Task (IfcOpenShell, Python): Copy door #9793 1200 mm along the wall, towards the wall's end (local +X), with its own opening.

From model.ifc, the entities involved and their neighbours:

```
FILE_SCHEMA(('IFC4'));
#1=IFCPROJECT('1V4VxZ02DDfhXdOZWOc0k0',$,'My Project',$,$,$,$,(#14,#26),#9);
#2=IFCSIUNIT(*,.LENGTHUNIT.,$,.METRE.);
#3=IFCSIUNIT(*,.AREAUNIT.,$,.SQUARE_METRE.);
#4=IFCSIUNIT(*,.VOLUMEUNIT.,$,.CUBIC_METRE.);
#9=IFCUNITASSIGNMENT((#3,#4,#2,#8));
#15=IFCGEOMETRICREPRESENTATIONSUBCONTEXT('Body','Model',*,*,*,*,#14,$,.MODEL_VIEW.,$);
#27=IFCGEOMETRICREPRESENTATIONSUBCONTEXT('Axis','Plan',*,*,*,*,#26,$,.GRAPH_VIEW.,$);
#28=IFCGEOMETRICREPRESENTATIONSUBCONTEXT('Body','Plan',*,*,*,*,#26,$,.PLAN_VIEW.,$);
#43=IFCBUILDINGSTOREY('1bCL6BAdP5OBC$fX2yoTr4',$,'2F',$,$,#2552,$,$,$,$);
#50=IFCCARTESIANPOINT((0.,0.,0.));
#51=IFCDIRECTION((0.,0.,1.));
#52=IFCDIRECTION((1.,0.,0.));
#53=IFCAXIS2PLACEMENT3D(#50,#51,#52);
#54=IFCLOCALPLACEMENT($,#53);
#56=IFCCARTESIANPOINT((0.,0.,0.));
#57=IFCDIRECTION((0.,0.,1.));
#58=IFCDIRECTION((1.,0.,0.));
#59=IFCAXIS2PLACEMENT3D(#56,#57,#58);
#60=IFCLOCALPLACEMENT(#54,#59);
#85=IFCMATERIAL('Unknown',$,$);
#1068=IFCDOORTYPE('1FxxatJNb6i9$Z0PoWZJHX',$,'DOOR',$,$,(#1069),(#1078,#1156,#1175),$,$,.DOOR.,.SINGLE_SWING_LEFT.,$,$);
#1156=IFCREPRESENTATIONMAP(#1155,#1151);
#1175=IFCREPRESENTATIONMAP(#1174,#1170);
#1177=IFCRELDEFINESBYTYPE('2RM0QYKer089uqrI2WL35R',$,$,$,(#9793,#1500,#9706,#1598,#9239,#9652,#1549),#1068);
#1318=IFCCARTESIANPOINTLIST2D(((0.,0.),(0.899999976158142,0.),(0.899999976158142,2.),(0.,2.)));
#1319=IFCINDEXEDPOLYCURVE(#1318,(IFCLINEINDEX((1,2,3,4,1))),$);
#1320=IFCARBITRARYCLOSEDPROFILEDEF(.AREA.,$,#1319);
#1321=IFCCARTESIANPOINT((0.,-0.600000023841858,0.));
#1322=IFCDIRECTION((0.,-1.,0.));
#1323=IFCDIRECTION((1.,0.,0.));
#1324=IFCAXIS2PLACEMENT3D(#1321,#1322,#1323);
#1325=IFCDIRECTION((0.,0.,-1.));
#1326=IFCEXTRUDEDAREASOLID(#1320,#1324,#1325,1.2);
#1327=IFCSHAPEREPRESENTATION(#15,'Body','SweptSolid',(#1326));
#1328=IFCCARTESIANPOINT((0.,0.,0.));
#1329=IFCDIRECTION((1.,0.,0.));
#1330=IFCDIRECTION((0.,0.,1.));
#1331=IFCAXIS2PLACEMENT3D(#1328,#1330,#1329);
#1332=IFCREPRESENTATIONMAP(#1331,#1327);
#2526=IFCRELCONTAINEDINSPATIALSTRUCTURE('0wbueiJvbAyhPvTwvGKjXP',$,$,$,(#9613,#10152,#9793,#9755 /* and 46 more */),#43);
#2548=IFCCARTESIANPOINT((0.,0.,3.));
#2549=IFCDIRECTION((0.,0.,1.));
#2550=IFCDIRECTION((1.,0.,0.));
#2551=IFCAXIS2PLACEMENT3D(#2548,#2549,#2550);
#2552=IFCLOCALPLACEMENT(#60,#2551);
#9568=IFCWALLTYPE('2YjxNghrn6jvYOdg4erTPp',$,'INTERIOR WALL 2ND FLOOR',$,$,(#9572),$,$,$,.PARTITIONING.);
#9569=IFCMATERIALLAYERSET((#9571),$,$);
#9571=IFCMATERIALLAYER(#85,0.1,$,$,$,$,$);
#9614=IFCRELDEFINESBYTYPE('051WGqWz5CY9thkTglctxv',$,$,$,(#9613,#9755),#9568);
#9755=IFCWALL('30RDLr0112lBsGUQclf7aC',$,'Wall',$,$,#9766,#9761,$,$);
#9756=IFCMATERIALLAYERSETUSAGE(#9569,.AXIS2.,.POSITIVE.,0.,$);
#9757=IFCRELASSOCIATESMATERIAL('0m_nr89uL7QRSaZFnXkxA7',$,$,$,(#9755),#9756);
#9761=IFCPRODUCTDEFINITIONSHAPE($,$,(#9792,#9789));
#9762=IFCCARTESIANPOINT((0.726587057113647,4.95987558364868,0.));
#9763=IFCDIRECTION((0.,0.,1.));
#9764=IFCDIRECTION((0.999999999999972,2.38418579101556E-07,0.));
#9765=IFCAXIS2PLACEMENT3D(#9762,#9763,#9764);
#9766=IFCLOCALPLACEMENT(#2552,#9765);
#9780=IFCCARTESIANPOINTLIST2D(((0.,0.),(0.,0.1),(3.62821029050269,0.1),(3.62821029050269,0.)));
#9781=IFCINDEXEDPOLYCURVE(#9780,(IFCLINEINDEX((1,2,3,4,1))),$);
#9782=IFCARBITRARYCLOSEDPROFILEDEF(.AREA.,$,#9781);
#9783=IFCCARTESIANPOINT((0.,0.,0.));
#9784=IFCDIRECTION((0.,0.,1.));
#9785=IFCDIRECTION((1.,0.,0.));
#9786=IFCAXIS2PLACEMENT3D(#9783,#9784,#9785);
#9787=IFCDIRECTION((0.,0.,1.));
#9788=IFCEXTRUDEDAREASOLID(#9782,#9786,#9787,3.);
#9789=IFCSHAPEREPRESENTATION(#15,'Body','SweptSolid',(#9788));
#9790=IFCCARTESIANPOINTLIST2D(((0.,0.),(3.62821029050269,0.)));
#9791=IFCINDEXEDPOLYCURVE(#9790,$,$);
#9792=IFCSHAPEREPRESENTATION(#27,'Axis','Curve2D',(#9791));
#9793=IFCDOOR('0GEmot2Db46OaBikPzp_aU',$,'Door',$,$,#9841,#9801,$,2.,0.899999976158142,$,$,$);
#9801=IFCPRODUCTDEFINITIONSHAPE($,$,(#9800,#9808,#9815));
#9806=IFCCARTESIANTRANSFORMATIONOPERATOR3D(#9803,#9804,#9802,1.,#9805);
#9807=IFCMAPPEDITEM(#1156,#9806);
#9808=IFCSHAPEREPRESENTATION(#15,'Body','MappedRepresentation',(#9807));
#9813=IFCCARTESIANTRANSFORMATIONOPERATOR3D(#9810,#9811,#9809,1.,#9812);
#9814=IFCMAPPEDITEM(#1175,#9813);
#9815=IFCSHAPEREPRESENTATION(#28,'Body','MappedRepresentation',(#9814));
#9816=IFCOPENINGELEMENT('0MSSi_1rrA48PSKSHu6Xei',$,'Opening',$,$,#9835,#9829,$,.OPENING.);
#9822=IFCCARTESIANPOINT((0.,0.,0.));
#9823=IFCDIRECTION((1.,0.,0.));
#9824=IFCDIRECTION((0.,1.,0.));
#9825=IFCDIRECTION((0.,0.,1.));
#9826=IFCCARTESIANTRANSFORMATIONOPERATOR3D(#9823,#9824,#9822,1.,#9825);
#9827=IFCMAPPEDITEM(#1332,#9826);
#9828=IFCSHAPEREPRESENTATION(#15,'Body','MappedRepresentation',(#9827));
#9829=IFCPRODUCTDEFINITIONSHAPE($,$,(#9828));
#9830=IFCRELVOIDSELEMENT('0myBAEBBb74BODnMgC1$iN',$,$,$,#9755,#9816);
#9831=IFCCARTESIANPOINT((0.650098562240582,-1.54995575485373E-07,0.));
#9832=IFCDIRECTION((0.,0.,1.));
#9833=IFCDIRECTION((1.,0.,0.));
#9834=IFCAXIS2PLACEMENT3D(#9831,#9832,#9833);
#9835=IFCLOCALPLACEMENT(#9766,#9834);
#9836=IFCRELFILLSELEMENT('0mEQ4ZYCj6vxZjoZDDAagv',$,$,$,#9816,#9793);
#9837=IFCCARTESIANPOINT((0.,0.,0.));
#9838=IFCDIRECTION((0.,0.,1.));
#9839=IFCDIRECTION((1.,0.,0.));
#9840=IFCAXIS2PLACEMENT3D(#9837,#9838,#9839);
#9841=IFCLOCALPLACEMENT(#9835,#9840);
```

```python
import ifcopenshell
import ifcopenshell.api.feature
import ifcopenshell.api.geometry
import ifcopenshell.api.root
import ifcopenshell.geom
import ifcopenshell.util.element
import ifcopenshell.util.placement
import ifcopenshell.util.shape

model = ifcopenshell.open("model.ifc")
settings = ifcopenshell.geom.settings()


def volume(element):
    """Net volume in cubic metres, openings subtracted."""
    shape = ifcopenshell.geom.create_shape(settings, element)
    return ifcopenshell.util.shape.get_volume(shape.geometry)


door = model.by_guid("0GEmot2Db46OaBikPzp_aU")
opening = door.FillsVoids[0].RelatingOpeningElement
wall = opening.VoidsElements[0].RelatingBuildingElement
before = volume(wall)
shift = ifcopenshell.util.placement.get_local_placement(wall.ObjectPlacement)[:3, 0] * 1.2

# copy_class copies the void relationship, type, container and properties, but no geometry.
new_opening = ifcopenshell.api.root.copy_class(model, product=opening)
new_opening.Representation = ifcopenshell.util.element.copy_deep(
    model, opening.Representation, exclude=["IfcGeometricRepresentationContext", "IfcRepresentationMap"]
)
new_door = ifcopenshell.api.root.copy_class(model, product=door)
new_door.Representation = ifcopenshell.util.element.copy_deep(
    model, door.Representation, exclude=["IfcGeometricRepresentationContext", "IfcRepresentationMap"]
)
ifcopenshell.api.feature.add_filling(model, opening=new_opening, element=new_door)

for old, new in ((opening, new_opening), (door, new_door)):
    matrix = ifcopenshell.util.placement.get_local_placement(old.ObjectPlacement)
    matrix[:3, 3] += shift
    ifcopenshell.api.geometry.edit_object_placement(model, product=new, matrix=matrix, is_si=False)

after = volume(wall)

print(f"wall volume {before:.3f} -> {after:.3f} m3")

model.write("model_updated.ifc")
```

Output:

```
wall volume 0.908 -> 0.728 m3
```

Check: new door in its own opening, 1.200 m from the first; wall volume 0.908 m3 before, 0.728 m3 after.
